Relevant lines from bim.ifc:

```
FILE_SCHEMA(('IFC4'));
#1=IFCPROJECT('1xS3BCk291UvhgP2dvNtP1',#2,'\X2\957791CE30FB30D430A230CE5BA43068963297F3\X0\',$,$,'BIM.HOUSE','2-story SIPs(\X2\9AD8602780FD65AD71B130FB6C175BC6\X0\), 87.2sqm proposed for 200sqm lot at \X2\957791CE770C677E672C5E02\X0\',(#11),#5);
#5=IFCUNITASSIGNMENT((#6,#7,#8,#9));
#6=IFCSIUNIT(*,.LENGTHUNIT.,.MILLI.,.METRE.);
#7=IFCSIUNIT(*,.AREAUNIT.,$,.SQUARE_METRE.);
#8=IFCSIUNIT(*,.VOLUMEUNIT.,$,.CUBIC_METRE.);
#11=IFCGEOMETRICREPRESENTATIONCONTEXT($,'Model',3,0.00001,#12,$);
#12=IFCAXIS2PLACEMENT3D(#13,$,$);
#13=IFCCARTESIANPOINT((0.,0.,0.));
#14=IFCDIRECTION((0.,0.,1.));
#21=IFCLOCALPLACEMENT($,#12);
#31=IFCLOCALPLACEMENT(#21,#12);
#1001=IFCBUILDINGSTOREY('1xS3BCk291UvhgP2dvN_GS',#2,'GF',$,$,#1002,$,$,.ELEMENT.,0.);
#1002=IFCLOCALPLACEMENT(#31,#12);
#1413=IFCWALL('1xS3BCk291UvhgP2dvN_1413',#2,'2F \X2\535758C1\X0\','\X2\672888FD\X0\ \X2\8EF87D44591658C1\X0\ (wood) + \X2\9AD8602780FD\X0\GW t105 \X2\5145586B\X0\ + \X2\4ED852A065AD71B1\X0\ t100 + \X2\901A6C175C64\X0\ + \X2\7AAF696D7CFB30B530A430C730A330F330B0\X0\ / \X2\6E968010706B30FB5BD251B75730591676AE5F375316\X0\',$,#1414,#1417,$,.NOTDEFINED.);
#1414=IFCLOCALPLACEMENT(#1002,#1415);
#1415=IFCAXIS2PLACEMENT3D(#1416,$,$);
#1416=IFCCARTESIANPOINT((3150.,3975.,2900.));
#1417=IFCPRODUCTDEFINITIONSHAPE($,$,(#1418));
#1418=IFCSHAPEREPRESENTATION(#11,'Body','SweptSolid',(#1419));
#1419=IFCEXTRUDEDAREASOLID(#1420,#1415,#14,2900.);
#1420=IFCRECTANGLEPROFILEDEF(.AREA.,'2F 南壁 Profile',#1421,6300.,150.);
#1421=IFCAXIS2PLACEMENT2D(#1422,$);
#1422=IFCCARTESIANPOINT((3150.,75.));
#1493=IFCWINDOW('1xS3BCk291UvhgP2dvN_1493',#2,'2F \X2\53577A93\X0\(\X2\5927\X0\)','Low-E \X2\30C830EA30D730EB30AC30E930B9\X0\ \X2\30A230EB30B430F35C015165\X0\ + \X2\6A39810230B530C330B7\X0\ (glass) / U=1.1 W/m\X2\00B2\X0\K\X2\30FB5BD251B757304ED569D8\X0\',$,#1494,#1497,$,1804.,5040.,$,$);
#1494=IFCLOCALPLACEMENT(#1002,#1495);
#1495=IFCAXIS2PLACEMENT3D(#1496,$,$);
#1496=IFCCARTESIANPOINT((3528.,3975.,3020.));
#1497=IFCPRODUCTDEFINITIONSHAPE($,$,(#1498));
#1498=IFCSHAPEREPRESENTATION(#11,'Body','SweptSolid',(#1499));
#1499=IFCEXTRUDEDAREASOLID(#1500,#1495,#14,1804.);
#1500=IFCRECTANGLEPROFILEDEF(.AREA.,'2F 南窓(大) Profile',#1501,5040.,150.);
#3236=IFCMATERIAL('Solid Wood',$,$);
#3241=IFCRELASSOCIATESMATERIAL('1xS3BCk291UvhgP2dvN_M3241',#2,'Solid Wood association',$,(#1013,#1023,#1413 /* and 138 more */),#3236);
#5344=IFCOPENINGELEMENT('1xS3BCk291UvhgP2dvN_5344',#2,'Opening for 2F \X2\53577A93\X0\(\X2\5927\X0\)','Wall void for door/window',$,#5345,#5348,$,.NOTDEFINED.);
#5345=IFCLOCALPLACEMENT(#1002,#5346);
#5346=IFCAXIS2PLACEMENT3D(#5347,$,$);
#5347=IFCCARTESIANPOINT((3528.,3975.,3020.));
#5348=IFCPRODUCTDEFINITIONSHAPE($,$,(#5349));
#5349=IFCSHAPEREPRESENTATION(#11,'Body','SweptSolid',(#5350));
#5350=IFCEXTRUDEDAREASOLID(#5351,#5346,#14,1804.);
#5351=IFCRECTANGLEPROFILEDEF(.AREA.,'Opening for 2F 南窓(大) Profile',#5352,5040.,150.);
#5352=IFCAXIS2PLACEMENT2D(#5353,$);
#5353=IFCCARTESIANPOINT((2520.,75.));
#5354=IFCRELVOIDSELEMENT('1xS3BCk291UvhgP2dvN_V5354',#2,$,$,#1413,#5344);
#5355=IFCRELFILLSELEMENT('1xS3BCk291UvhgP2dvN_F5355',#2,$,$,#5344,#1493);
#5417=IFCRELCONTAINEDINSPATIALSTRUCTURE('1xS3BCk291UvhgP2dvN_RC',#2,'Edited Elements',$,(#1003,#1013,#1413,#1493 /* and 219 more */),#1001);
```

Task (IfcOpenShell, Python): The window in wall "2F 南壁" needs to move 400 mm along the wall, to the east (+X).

```python
import ifcopenshell
import ifcopenshell.api.geometry
import ifcopenshell.util.placement

model = ifcopenshell.open("bim.ifc")

window = model.by_guid("1xS3BCk291UvhgP2dvN_1493")
opening = window.FillsVoids[0].RelatingOpeningElement
wall = opening.VoidsElements[0].RelatingBuildingElement

wall_matrix = ifcopenshell.util.placement.get_local_placement(wall.ObjectPlacement)
shift = wall_matrix[:3, 0] * 400.0
before = ifcopenshell.util.placement.get_local_placement(window.ObjectPlacement)[:3, 3].copy()

# The window is not placed relative to its opening, so move both.
for product in (opening, window):
    matrix = ifcopenshell.util.placement.get_local_placement(product.ObjectPlacement)
    matrix[:3, 3] += shift
    ifcopenshell.api.geometry.edit_object_placement(model, product=product, matrix=matrix, is_si=False)

after = ifcopenshell.util.placement.get_local_placement(window.ObjectPlacement)[:3, 3]
print("window moved by", (after - before).round(3) + 0.0)

model.write("bim_v2.ifc")
```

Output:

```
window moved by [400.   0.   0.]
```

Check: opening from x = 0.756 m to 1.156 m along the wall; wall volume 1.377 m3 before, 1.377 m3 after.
